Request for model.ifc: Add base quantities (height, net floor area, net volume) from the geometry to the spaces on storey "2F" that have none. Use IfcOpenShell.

First a look at what the model holds.

```python
import ifcopenshell
import ifcopenshell.util.element
import ifcopenshell.util.unit

model = ifcopenshell.open("model.ifc")
print(model.schema)
for unit_type in ("LENGTHUNIT", "AREAUNIT", "VOLUMEUNIT"):
    print(unit_type, ifcopenshell.util.unit.calculate_unit_scale(model, unit_type))
storey = next(s for s in model.by_type("IfcBuildingStorey") if s.Name == "2F")
spaces = [e for e in ifcopenshell.util.element.get_decomposition(storey) if e.is_a("IfcSpace")]
for e in sorted(spaces, key=lambda e: e.id()):
    print(e.id(), e.is_a(), e.Name, list(ifcopenshell.util.element.get_psets(e, qtos_only=True)), sep=" | ")
```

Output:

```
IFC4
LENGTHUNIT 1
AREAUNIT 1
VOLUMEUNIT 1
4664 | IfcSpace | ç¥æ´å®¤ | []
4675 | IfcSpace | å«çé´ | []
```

```python
import ifcopenshell
import ifcopenshell.api.pset
import ifcopenshell.geom
import ifcopenshell.util.element
import ifcopenshell.util.shape
import ifcopenshell.util.unit

model = ifcopenshell.open("model.ifc")
unit_scale = ifcopenshell.util.unit.calculate_unit_scale(model)
area_scale = ifcopenshell.util.unit.calculate_unit_scale(model, "AREAUNIT")
volume_scale = ifcopenshell.util.unit.calculate_unit_scale(model, "VOLUMEUNIT")
settings = ifcopenshell.geom.settings()

storey = next(s for s in model.by_type("IfcBuildingStorey") if s.Name == "2F")
spaces = [e for e in ifcopenshell.util.element.get_decomposition(storey) if e.is_a("IfcSpace")]

for e in sorted(spaces, key=lambda e: e.id()):
    if ifcopenshell.util.element.get_psets(e, qtos_only=True, should_inherit=False):
        continue
    # Geometry comes back in metres, in the element's own axes.
    shape = ifcopenshell.geom.create_shape(settings, e)
    values = {
        "Height": ifcopenshell.util.shape.get_z(shape.geometry) / unit_scale,
        "NetFloorArea": ifcopenshell.util.shape.get_footprint_area(shape.geometry) / area_scale,
        "NetVolume": ifcopenshell.util.shape.get_volume(shape.geometry) / volume_scale,
    }
    qto = ifcopenshell.api.pset.add_qto(model, product=e, name="Qto_SpaceBaseQuantities")
    ifcopenshell.api.pset.edit_qto(model, qto=qto, properties=values)
    print(e.id(), {k: round(v, 3) for k, v in values.items()})

model.write("model_v2.ifc")
```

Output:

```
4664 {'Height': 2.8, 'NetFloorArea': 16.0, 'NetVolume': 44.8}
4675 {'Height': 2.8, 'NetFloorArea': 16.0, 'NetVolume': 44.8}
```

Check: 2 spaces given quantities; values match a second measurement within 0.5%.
